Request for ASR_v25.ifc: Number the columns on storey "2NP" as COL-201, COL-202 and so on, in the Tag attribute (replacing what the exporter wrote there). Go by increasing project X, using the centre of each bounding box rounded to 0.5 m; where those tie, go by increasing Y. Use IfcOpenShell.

First a look at what the model holds.

```python
import ifcopenshell
import ifcopenshell.util.element
import ifcopenshell.util.placement

model = ifcopenshell.open("ASR_v25.ifc")
print(model.schema)
storey = next(s for s in model.by_type("IfcBuildingStorey") if s.Name == "2NP")
columns = [e for e in ifcopenshell.util.element.get_decomposition(storey) if e.is_a("IfcColumn")]
for e in sorted(columns, key=lambda e: e.id()):
    origin = ifcopenshell.util.placement.get_local_placement(e.ObjectPlacement)[:3, 3]
    print(e.id(), e.Tag, e.Name, origin.round(2) + 0.0, sep=" | ")
```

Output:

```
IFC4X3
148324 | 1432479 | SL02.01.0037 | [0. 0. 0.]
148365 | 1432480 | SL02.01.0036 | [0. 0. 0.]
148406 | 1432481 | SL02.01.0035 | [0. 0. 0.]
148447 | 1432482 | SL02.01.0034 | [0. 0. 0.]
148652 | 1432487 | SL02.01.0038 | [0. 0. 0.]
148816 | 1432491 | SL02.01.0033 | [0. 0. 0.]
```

```python
import ifcopenshell
import ifcopenshell.geom
import ifcopenshell.util.element
import ifcopenshell.util.shape

model = ifcopenshell.open("ASR_v25.ifc")
settings = ifcopenshell.geom.settings()
settings.set("use-world-coords", True)


def centre(element):
    shape = ifcopenshell.geom.create_shape(settings, element)
    return ifcopenshell.util.shape.get_bbox_centroid(shape.geometry)


storey = next(s for s in model.by_type("IfcBuildingStorey") if s.Name == "2NP")
columns = [e for e in ifcopenshell.util.element.get_decomposition(storey) if e.is_a("IfcColumn")]

# Insertion points can sit at a corner or the storey origin, so sort by the geometry (in metres).
centres = {e: centre(e) for e in columns}
columns.sort(key=lambda e: (round(centres[e][0] / 0.5), centres[e][1]))

for i, e in enumerate(columns, start=1):
    number = f"COL-2{i:02d}"
    e.Tag = number
    print(e.id(), number)

model.write("ASR_v25_rev.ifc")
```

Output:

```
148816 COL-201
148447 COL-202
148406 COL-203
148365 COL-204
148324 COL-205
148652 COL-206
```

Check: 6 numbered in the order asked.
